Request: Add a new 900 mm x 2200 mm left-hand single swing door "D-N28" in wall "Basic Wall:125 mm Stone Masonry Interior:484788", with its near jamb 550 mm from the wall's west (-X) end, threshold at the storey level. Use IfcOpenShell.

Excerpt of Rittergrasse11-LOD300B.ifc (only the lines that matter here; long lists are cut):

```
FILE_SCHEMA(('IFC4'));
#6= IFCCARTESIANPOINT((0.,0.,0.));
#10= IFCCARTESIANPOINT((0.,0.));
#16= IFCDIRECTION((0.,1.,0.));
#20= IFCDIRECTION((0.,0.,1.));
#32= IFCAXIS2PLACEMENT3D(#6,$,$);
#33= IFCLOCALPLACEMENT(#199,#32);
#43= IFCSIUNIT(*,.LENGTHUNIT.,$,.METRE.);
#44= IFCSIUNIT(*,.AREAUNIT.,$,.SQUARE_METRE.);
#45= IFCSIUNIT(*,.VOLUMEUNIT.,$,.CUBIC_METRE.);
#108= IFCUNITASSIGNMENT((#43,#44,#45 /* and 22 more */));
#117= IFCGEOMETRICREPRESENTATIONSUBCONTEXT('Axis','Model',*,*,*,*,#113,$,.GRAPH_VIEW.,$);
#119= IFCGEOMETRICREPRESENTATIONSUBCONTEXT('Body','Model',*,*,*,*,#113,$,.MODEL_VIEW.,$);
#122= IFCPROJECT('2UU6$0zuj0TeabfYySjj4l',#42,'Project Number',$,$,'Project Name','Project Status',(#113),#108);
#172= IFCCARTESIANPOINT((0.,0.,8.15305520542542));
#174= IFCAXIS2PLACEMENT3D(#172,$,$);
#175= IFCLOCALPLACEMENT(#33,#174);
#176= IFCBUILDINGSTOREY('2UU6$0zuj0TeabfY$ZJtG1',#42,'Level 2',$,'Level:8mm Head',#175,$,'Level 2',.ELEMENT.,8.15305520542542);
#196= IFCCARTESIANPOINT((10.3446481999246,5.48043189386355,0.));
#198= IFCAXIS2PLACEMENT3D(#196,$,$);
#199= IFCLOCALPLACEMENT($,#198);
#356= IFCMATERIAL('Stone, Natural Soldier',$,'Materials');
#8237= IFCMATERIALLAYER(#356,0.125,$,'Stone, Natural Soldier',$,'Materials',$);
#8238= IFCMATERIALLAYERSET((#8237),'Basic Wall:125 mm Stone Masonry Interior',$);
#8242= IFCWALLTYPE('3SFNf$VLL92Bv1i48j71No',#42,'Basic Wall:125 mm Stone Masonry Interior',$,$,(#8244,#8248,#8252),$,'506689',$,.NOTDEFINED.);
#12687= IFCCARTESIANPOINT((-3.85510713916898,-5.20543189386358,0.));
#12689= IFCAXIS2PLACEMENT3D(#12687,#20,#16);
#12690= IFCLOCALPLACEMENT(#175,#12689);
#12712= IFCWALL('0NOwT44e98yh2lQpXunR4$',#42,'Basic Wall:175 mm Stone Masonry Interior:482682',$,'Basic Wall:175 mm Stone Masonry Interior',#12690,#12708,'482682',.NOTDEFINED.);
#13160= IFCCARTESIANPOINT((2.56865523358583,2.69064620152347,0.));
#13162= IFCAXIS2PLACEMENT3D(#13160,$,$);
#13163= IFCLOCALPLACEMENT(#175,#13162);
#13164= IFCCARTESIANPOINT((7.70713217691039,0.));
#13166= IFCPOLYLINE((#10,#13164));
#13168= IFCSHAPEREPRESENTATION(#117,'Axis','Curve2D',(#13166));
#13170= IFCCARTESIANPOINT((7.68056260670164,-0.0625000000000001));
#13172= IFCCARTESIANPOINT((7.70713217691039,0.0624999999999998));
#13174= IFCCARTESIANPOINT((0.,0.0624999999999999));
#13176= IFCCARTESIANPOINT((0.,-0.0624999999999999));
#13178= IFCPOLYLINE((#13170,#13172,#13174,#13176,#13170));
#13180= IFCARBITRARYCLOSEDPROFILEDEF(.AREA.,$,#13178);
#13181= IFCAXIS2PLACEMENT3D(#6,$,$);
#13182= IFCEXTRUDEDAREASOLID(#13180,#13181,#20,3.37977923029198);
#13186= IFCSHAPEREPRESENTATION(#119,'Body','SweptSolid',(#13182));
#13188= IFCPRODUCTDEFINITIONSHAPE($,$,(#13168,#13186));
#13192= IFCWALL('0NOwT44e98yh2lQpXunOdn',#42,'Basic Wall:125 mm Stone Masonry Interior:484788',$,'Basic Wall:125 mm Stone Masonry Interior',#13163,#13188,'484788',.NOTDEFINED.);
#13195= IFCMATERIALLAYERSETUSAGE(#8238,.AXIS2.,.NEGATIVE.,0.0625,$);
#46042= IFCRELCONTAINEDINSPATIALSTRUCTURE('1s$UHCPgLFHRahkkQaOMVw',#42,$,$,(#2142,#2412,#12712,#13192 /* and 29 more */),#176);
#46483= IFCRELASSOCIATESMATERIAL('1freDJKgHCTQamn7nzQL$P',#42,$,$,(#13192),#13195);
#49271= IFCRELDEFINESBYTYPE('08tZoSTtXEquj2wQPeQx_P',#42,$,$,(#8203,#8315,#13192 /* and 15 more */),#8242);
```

```python
import numpy as np
import ifcopenshell
import ifcopenshell.api.feature
import ifcopenshell.api.geometry
import ifcopenshell.api.root
import ifcopenshell.api.spatial
import ifcopenshell.geom
import ifcopenshell.util.element
import ifcopenshell.util.placement
import ifcopenshell.util.representation
import ifcopenshell.util.shape
import ifcopenshell.util.unit

model = ifcopenshell.open("Rittergrasse11-LOD300B.ifc")
unit_scale = ifcopenshell.util.unit.calculate_unit_scale(model)
settings = ifcopenshell.geom.settings()


def volume(element):
    """Net volume in cubic metres, openings subtracted."""
    shape = ifcopenshell.geom.create_shape(settings, element)
    return ifcopenshell.util.shape.get_volume(shape.geometry)


wall = model.by_id(13192)
storey = ifcopenshell.util.element.get_container(wall, ifc_class="IfcBuildingStorey")
context = ifcopenshell.util.representation.get_context(model, "Model", "Body", "MODEL_VIEW")
before = volume(wall)

width, height, from_end, sill = 0.9, 2.2, 0.55, 0.0  # metres

# The wall runs along its own X axis, and the end named is its -X end.
wall_shape = ifcopenshell.geom.create_shape(settings, wall)
x, y, z = ifcopenshell.util.shape.get_vertices(wall_shape.geometry).T
start = x.min() + from_end
face, thickness = float(y.min()), float(y.max() - y.min())
wall_matrix = ifcopenshell.util.placement.get_local_placement(wall.ObjectPlacement)
level = ifcopenshell.util.placement.get_local_placement(storey.ObjectPlacement)[2, 3]


def in_wall(x, y):
    """Placement at x, y metres in the wall's axes, at sill height."""
    matrix = wall_matrix.copy()
    matrix[:, 3] = wall_matrix @ np.array([x / unit_scale, y / unit_scale, 0.0, 1.0])
    matrix[2, 3] = level + sill / unit_scale
    return matrix


# Opening: a box that overshoots both wall faces by 50 mm.
opening = ifcopenshell.api.root.create_entity(model, ifc_class="IfcOpeningElement", predefined_type="OPENING")
box = ifcopenshell.api.geometry.add_wall_representation(
    model, context=context, length=width, height=height, thickness=thickness + 0.1
)
ifcopenshell.api.geometry.assign_representation(model, product=opening, representation=box)
ifcopenshell.api.geometry.edit_object_placement(model, product=opening, matrix=in_wall(start, face - 0.05), is_si=False)
ifcopenshell.api.feature.add_feature(model, feature=opening, element=wall)

door = ifcopenshell.api.root.create_entity(model, ifc_class="IfcDoor", name="D-N28", predefined_type="DOOR")
door.OverallWidth, door.OverallHeight = width / unit_scale, height / unit_scale
door.OperationType = "SINGLE_SWING_LEFT"
body = ifcopenshell.api.geometry.add_door_representation(
    model,
    context=context,
    overall_width=door.OverallWidth,
    overall_height=door.OverallHeight,
    operation_type="SINGLE_SWING_LEFT",
    lining_properties={"LiningDepth": thickness / unit_scale, "ThresholdDepth": thickness / unit_scale},
)
ifcopenshell.api.geometry.assign_representation(model, product=door, representation=body)
ifcopenshell.api.spatial.assign_container(model, products=[door], relating_structure=storey)
ifcopenshell.api.feature.add_filling(model, opening=opening, element=door)

# The lining spans the wall, so the door starts at the wall face.
ifcopenshell.api.geometry.edit_object_placement(model, product=door, matrix=in_wall(start, face), is_si=False)

after = volume(wall)

print(f"wall volume {before:.3f} -> {after:.3f} m3")

model.write("Rittergrasse11-LOD300B_edited.ifc")
```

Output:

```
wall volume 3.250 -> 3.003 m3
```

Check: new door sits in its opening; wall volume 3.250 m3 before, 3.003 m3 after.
